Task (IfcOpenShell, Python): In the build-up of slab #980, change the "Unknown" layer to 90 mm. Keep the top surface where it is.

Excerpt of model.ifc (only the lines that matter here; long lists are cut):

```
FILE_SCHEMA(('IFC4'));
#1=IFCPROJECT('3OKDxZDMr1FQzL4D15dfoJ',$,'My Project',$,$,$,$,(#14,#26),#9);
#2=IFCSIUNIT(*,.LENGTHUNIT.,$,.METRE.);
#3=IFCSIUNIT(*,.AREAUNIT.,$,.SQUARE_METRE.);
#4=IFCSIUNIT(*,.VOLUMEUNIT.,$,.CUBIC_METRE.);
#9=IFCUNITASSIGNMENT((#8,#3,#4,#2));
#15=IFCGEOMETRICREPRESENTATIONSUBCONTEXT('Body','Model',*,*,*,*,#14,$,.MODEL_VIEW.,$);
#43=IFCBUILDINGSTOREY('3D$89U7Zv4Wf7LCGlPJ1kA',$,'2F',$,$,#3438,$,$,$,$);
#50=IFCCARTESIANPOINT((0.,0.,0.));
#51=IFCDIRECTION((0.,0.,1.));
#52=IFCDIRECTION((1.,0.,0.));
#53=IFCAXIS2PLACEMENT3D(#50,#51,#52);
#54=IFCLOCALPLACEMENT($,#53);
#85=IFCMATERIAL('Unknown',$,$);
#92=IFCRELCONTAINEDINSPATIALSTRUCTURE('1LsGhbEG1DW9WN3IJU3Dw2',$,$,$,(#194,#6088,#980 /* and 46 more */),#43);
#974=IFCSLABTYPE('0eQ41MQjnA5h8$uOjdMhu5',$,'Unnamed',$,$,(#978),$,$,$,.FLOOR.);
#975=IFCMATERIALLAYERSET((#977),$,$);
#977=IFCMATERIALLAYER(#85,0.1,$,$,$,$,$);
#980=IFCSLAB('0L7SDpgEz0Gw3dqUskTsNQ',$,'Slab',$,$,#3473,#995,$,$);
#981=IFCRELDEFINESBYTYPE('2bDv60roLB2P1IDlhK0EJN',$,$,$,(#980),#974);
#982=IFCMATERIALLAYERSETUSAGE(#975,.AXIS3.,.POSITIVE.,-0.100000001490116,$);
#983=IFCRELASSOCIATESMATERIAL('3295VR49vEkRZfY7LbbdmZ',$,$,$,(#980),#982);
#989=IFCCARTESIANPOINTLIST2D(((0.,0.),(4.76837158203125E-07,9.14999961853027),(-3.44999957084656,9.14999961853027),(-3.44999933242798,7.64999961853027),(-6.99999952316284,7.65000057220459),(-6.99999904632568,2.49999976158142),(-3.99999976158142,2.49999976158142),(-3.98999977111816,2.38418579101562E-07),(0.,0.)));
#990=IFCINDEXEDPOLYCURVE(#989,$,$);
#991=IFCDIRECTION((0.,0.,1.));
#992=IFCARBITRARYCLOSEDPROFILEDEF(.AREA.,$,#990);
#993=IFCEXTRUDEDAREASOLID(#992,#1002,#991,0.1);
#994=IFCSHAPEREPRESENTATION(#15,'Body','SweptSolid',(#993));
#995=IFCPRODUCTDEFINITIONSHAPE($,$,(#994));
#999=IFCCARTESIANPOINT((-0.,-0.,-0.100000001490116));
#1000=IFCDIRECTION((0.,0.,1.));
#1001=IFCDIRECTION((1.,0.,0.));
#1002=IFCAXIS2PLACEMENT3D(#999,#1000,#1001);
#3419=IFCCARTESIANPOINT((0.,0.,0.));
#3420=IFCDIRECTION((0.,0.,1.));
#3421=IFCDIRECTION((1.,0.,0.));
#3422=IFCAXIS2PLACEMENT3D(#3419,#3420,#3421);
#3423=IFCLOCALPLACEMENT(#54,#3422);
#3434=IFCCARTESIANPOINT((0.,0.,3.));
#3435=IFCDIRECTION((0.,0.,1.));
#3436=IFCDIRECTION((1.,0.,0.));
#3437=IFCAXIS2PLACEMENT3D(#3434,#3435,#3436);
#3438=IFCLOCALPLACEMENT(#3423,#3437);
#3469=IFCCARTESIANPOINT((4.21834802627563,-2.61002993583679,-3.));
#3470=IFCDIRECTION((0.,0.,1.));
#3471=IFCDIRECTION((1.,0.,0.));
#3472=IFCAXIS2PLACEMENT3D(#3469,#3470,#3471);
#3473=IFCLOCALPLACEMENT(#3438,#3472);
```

```python
import ifcopenshell
import ifcopenshell.util.element
import ifcopenshell.util.representation
import ifcopenshell.util.unit

model = ifcopenshell.open("model.ifc")
unit_scale = ifcopenshell.util.unit.calculate_unit_scale(model)

layer_set = model.by_id(975)
layer = next(l for l in layer_set.MaterialLayers if l.Material and l.Material.Name == "Unknown")
change = 0.09 / unit_scale - layer.LayerThickness
layer.LayerThickness += change

# Geometry does not follow the layer set by itself.
slabs = [e for e in ifcopenshell.util.element.get_elements_by_material(model, layer_set) if e.is_a("IfcSlab")]
for slab in sorted(slabs, key=lambda e: e.id()):
    body = ifcopenshell.util.representation.get_representation(slab, "Model", "Body")
    solid = body.Items[0]
    old_depth = solid.Depth
    solid.Depth += change
    # Extruded upwards: lower the start of the extrusion so the top stays.
    x, y, z = solid.Position.Location.Coordinates
    solid.Position.Location = model.createIfcCartesianPoint((x, y, z - change))
    print(slab.id(), f"{old_depth:g} -> {solid.Depth:g}")

# The layers are counted up from the underside, which has moved.
for usage in {ifcopenshell.util.element.get_material(slab) for slab in slabs}:
    usage.OffsetFromReferenceLine -= change

model.write("model_updated.ifc")
```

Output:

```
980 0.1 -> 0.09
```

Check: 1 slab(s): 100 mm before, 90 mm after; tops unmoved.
